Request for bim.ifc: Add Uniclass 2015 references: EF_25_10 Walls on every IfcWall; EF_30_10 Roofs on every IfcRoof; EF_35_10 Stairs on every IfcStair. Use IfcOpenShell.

First a look at what the model holds.

```python
import ifcopenshell

model = ifcopenshell.open("bim.ifc")
print(model.schema)
print("classifications:", [c.Name for c in model.by_type("IfcClassification")])
for ifc_class in ("IfcDoor", "IfcRoof", "IfcStair", "IfcWall", "IfcWindow"):
    print(ifc_class, len(model.by_type(ifc_class)))
```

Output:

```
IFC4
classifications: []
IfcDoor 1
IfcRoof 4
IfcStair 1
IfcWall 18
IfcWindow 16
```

```python
import ifcopenshell
import ifcopenshell.api.classification

model = ifcopenshell.open("bim.ifc")

system = ifcopenshell.api.classification.add_classification(model, classification="Uniclass 2015")

codes = {
    "IfcWall": ("EF_25_10", "Walls"),
    "IfcRoof": ("EF_30_10", "Roofs"),
    "IfcStair": ("EF_35_10", "Stairs"),
}
for ifc_class, (code, name) in codes.items():
    products = model.by_type(ifc_class)
    ifcopenshell.api.classification.add_reference(
        model, products=products, classification=system, identification=code, name=name
    )
    print(code, len(products))

model.write("bim_updated.ifc")
```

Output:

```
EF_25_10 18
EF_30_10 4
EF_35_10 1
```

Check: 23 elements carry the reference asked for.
